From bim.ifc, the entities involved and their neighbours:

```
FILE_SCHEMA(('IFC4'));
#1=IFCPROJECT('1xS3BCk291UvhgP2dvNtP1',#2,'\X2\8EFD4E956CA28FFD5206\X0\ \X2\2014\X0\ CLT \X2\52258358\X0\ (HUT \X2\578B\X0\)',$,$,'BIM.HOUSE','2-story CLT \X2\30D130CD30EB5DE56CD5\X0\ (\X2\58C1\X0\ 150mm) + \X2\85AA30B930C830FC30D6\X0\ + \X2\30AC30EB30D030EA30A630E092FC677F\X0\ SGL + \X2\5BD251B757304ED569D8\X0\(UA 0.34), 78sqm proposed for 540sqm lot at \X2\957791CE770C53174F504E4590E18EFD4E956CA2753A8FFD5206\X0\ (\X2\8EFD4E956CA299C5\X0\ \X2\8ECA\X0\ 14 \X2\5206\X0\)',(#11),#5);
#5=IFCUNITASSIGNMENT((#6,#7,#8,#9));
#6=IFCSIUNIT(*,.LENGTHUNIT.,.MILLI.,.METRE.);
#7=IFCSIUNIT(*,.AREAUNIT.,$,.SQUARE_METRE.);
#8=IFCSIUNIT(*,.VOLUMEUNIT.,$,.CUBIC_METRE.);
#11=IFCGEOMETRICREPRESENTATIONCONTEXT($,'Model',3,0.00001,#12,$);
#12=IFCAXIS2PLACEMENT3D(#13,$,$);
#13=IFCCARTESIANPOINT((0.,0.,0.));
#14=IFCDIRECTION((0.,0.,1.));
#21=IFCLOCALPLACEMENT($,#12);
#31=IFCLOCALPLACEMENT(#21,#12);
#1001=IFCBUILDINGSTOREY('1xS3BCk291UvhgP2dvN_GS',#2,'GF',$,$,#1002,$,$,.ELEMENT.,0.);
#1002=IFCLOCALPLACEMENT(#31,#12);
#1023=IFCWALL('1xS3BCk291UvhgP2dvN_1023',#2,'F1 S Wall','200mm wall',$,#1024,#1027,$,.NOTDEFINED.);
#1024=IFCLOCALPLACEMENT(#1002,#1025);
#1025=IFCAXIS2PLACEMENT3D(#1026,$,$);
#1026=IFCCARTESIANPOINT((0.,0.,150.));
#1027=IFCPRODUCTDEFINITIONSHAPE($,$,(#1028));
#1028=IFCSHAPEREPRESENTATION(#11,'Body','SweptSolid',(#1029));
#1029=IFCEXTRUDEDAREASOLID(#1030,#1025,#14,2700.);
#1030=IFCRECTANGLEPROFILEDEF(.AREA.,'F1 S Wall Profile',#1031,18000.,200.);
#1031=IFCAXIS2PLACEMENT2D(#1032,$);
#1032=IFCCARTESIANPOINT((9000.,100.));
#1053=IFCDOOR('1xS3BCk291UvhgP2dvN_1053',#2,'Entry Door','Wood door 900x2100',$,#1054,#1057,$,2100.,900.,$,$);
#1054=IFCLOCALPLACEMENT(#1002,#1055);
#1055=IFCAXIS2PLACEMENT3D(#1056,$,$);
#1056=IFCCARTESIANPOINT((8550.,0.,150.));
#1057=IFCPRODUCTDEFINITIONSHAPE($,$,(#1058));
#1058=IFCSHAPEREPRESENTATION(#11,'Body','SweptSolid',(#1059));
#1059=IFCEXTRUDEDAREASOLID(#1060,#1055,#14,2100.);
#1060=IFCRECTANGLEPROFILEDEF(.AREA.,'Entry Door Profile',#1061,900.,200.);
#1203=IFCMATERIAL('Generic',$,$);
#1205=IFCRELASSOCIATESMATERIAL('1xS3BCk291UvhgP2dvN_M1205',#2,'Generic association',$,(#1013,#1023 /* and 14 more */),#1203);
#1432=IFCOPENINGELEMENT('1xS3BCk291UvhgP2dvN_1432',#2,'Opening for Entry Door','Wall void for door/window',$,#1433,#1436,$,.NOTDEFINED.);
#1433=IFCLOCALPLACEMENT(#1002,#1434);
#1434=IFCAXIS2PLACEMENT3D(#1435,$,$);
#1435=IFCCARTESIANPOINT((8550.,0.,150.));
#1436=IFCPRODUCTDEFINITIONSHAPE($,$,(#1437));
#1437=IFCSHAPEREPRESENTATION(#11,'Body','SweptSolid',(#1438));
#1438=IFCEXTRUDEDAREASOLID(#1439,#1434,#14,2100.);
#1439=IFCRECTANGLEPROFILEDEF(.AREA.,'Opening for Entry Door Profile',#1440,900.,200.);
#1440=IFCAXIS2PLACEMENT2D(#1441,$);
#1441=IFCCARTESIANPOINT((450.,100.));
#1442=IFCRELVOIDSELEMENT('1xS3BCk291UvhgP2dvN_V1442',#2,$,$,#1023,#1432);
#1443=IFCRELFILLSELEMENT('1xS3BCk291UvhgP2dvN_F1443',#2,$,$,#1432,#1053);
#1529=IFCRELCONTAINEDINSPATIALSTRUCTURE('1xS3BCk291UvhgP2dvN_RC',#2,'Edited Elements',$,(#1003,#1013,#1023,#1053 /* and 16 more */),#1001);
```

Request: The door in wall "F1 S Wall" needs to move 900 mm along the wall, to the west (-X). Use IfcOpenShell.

```python
import ifcopenshell
import ifcopenshell.api.geometry
import ifcopenshell.util.placement

model = ifcopenshell.open("bim.ifc")

door = model.by_guid("1xS3BCk291UvhgP2dvN_1053")
opening = door.FillsVoids[0].RelatingOpeningElement
wall = opening.VoidsElements[0].RelatingBuildingElement

wall_matrix = ifcopenshell.util.placement.get_local_placement(wall.ObjectPlacement)
shift = wall_matrix[:3, 0] * -900.0
before = ifcopenshell.util.placement.get_local_placement(door.ObjectPlacement)[:3, 3].copy()

# The door is not placed relative to its opening, so move both.
for product in (opening, door):
    matrix = ifcopenshell.util.placement.get_local_placement(product.ObjectPlacement)
    matrix[:3, 3] += shift
    ifcopenshell.api.geometry.edit_object_placement(model, product=product, matrix=matrix, is_si=False)

after = ifcopenshell.util.placement.get_local_placement(door.ObjectPlacement)[:3, 3]
print("door moved by", (after - before).round(3) + 0.0)

model.write("bim_rev.ifc")
```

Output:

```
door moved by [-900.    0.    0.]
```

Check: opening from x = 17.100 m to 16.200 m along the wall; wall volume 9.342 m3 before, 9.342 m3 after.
